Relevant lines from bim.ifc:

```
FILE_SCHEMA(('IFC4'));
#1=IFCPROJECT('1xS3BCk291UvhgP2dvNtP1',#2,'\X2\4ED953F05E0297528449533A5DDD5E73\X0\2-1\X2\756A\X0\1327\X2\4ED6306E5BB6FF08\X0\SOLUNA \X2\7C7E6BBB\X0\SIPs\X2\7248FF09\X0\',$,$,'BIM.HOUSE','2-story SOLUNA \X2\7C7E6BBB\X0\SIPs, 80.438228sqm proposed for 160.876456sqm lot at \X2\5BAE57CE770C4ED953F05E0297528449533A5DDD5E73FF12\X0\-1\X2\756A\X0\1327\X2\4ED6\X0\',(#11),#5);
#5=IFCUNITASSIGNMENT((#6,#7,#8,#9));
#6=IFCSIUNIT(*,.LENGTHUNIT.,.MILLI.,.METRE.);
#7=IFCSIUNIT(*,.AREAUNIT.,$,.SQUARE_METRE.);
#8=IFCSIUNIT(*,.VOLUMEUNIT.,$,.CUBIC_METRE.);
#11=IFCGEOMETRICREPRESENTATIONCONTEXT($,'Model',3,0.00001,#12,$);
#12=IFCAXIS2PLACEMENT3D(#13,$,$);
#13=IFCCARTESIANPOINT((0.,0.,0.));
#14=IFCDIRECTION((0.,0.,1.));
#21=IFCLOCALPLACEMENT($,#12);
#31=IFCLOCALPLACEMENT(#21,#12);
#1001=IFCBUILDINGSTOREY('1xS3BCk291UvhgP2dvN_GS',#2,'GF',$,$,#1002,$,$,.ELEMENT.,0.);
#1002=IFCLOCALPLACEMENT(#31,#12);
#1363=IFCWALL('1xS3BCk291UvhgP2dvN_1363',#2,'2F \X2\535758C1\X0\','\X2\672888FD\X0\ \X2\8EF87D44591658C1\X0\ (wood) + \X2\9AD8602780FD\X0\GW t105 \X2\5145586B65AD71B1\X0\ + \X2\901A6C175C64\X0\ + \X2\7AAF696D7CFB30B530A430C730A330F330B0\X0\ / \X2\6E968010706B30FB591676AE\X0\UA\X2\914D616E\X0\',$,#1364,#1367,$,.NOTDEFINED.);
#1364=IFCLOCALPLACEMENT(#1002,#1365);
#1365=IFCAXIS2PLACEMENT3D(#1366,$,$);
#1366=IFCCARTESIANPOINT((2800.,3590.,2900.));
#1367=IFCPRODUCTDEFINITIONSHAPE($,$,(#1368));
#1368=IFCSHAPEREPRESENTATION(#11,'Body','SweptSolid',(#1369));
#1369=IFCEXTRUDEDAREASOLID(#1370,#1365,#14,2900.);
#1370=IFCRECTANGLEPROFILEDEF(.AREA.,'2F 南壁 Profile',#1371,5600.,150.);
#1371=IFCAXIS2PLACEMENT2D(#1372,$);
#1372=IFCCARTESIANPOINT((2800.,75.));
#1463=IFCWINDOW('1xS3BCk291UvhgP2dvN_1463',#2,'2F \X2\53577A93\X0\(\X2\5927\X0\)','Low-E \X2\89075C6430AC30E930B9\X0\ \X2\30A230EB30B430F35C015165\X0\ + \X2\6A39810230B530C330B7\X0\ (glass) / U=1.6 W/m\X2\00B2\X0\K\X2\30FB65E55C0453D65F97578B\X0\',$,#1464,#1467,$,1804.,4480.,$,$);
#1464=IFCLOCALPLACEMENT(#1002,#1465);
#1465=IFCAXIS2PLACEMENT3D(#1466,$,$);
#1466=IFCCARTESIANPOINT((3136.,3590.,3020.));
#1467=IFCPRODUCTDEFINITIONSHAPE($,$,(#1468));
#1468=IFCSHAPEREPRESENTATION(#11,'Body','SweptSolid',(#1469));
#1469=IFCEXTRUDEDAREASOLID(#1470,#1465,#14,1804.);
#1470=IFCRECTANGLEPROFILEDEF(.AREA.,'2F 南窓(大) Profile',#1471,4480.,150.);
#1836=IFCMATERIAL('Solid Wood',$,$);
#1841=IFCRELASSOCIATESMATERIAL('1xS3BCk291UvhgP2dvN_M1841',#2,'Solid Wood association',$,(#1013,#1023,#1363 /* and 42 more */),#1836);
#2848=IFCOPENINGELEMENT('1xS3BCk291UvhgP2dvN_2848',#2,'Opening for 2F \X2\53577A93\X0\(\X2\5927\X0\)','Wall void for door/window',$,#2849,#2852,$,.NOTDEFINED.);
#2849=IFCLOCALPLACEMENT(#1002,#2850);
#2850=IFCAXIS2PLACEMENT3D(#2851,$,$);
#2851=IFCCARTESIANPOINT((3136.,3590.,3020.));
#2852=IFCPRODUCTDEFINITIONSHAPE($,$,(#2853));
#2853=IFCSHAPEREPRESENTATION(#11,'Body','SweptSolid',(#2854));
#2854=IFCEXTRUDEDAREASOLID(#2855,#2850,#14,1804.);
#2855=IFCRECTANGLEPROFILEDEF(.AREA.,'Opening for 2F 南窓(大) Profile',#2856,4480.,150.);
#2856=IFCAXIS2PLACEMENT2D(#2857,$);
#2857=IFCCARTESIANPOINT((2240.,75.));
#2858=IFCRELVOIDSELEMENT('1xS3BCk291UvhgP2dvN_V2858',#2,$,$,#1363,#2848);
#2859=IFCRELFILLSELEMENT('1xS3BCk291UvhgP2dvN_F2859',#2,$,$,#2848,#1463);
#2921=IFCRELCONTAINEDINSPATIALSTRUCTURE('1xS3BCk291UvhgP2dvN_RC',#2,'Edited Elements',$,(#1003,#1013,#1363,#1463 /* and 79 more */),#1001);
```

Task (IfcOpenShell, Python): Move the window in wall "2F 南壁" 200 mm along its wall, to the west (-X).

```python
import ifcopenshell
import ifcopenshell.api.geometry
import ifcopenshell.util.placement

model = ifcopenshell.open("bim.ifc")

window = model.by_id(1463)
opening = window.FillsVoids[0].RelatingOpeningElement
wall = opening.VoidsElements[0].RelatingBuildingElement

wall_matrix = ifcopenshell.util.placement.get_local_placement(wall.ObjectPlacement)
shift = wall_matrix[:3, 0] * -200.0
before = ifcopenshell.util.placement.get_local_placement(window.ObjectPlacement)[:3, 3].copy()

# The window is not placed relative to its opening, so move both.
for product in (opening, window):
    matrix = ifcopenshell.util.placement.get_local_placement(product.ObjectPlacement)
    matrix[:3, 3] += shift
    ifcopenshell.api.geometry.edit_object_placement(model, product=product, matrix=matrix, is_si=False)

after = ifcopenshell.util.placement.get_local_placement(window.ObjectPlacement)[:3, 3]
print("window moved by", (after - before).round(3) + 0.0)

model.write("bim_v2.ifc")
```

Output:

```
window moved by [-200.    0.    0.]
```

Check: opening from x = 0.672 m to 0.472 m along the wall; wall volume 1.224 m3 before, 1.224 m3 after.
